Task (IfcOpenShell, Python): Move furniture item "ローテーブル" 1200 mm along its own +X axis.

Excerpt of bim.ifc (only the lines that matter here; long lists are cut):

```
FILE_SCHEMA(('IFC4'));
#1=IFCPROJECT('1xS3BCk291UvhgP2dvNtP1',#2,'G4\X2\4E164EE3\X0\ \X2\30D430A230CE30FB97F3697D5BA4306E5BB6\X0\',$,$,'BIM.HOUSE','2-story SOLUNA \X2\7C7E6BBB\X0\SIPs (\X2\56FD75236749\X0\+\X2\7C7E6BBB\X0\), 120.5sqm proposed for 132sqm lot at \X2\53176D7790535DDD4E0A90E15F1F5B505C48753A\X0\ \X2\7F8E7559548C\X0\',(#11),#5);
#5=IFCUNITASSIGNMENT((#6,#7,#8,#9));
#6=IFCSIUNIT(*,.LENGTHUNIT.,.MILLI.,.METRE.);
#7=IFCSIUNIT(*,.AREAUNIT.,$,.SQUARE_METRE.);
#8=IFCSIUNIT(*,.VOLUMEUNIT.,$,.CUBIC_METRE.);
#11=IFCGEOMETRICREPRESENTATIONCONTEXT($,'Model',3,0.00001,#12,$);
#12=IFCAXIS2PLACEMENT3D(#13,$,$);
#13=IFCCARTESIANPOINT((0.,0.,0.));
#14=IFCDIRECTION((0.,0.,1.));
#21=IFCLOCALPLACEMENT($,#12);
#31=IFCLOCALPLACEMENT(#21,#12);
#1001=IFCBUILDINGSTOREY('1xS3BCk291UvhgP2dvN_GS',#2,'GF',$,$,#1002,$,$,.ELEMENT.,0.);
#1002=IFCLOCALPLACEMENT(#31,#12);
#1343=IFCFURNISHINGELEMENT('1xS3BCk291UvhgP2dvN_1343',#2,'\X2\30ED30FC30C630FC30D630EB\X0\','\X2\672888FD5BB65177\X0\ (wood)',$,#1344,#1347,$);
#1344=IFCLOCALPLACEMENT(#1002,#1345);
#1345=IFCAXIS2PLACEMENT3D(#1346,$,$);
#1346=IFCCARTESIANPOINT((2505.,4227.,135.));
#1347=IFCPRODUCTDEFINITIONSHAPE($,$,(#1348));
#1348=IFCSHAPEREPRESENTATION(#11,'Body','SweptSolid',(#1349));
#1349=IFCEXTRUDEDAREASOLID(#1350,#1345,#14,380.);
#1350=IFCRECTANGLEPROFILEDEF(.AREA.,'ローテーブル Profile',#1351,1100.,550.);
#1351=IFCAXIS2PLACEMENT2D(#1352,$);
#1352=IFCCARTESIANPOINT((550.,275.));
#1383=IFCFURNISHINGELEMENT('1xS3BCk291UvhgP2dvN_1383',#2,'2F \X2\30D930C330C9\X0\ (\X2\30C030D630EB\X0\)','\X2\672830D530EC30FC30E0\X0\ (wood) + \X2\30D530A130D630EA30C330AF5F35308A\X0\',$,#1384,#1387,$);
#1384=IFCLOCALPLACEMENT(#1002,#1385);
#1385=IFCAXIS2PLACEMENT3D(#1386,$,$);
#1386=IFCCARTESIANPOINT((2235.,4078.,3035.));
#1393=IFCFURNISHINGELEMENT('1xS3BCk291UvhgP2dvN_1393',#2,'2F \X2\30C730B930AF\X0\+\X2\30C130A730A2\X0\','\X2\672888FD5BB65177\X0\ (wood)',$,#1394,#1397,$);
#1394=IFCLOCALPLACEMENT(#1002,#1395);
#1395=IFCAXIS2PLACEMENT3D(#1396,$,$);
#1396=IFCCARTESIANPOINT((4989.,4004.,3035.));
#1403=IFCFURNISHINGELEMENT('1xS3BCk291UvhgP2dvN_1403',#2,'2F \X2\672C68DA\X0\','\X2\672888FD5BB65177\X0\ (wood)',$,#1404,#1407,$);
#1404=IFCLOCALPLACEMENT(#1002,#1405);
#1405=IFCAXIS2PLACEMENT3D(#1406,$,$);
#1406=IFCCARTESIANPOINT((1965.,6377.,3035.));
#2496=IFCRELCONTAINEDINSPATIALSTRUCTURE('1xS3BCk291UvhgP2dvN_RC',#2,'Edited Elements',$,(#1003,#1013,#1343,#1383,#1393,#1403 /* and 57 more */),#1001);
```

```python
import ifcopenshell
import ifcopenshell.api.geometry
import ifcopenshell.util.placement

model = ifcopenshell.open("bim.ifc")

item = model.by_guid("1xS3BCk291UvhgP2dvN_1343")
matrix = ifcopenshell.util.placement.get_local_placement(item.ObjectPlacement)
matrix[:3, 3] += matrix[:3, 0] * 1200.0
ifcopenshell.api.geometry.edit_object_placement(model, product=item, matrix=matrix, is_si=False)

print(ifcopenshell.util.placement.get_local_placement(item.ObjectPlacement).round(3) + 0.0)

model.write("bim_rev.ifc")
```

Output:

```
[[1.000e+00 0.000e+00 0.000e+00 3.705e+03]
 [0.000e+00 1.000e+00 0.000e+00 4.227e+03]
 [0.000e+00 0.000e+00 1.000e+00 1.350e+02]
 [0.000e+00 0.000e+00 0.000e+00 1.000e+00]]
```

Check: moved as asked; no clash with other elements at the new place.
